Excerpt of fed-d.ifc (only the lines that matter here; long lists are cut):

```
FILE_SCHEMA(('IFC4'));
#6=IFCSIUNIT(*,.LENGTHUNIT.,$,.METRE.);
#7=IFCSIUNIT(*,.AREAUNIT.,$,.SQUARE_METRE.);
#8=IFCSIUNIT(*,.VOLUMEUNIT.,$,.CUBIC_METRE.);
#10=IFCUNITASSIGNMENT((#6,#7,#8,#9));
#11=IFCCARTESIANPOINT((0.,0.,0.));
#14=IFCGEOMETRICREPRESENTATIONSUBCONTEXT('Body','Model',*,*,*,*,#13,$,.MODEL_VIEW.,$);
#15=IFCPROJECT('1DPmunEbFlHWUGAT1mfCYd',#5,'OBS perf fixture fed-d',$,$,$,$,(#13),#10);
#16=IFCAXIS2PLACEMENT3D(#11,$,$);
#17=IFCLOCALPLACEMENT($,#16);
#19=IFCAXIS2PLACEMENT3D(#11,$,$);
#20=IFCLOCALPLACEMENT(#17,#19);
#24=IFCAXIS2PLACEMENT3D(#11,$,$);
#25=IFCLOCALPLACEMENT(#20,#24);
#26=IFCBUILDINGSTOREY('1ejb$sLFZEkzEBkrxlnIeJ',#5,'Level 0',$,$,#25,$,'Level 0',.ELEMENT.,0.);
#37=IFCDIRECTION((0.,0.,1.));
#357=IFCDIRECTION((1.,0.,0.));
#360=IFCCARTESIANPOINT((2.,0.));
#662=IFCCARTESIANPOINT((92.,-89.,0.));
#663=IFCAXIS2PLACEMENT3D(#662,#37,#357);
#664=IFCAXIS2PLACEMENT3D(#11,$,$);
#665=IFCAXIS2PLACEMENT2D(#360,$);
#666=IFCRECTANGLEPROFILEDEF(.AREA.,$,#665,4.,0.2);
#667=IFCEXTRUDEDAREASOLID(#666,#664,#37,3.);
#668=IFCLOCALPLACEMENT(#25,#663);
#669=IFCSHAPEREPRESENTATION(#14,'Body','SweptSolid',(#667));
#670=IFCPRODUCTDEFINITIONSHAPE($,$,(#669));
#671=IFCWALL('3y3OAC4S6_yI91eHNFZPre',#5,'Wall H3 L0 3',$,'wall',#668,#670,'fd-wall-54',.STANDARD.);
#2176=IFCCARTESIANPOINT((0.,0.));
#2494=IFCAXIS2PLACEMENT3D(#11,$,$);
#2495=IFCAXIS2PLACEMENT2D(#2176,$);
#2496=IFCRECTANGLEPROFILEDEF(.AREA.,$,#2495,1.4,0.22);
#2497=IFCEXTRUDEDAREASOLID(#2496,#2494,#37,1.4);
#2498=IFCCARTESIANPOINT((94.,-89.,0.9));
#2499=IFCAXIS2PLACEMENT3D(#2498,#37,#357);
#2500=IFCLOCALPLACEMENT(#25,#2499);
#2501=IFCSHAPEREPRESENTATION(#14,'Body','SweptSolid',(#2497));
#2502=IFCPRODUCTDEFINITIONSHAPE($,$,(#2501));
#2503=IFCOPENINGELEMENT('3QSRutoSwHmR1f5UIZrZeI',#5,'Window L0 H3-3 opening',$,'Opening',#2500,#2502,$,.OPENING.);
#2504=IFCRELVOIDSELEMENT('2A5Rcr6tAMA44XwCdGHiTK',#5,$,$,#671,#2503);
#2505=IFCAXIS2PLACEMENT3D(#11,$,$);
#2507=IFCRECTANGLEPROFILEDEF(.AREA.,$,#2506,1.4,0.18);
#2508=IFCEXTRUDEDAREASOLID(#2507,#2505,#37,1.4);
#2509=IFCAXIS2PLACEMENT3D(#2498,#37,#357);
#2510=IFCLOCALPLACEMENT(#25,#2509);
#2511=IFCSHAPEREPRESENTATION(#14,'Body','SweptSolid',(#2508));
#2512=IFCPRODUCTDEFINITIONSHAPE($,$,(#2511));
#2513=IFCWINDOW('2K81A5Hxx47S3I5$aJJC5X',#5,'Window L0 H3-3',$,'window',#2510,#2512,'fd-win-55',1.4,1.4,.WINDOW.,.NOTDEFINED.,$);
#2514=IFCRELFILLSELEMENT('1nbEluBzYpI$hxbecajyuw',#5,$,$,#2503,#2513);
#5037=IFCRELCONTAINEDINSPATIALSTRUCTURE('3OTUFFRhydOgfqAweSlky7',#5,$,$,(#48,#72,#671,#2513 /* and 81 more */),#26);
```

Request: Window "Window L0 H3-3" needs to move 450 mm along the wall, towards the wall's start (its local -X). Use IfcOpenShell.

```python
import ifcopenshell
import ifcopenshell.api.geometry
import ifcopenshell.util.placement
import ifcopenshell.util.unit

model = ifcopenshell.open("fed-d.ifc")
unit_scale = ifcopenshell.util.unit.calculate_unit_scale(model)

window = model.by_guid("2K81A5Hxx47S3I5$aJJC5X")
opening = window.FillsVoids[0].RelatingOpeningElement
wall = opening.VoidsElements[0].RelatingBuildingElement

wall_matrix = ifcopenshell.util.placement.get_local_placement(wall.ObjectPlacement)
shift = wall_matrix[:3, 0] * -0.45 / unit_scale
before = ifcopenshell.util.placement.get_local_placement(window.ObjectPlacement)[:3, 3].copy()

# The window is not placed relative to its opening, so move both.
for product in (opening, window):
    matrix = ifcopenshell.util.placement.get_local_placement(product.ObjectPlacement)
    matrix[:3, 3] += shift
    ifcopenshell.api.geometry.edit_object_placement(model, product=product, matrix=matrix, is_si=False)

after = ifcopenshell.util.placement.get_local_placement(window.ObjectPlacement)[:3, 3]
print("window moved by", (after - before).round(3) + 0.0)

model.write("fed-d_edited.ifc")
```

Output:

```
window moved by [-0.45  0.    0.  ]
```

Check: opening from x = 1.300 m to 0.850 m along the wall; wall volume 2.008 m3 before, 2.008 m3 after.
